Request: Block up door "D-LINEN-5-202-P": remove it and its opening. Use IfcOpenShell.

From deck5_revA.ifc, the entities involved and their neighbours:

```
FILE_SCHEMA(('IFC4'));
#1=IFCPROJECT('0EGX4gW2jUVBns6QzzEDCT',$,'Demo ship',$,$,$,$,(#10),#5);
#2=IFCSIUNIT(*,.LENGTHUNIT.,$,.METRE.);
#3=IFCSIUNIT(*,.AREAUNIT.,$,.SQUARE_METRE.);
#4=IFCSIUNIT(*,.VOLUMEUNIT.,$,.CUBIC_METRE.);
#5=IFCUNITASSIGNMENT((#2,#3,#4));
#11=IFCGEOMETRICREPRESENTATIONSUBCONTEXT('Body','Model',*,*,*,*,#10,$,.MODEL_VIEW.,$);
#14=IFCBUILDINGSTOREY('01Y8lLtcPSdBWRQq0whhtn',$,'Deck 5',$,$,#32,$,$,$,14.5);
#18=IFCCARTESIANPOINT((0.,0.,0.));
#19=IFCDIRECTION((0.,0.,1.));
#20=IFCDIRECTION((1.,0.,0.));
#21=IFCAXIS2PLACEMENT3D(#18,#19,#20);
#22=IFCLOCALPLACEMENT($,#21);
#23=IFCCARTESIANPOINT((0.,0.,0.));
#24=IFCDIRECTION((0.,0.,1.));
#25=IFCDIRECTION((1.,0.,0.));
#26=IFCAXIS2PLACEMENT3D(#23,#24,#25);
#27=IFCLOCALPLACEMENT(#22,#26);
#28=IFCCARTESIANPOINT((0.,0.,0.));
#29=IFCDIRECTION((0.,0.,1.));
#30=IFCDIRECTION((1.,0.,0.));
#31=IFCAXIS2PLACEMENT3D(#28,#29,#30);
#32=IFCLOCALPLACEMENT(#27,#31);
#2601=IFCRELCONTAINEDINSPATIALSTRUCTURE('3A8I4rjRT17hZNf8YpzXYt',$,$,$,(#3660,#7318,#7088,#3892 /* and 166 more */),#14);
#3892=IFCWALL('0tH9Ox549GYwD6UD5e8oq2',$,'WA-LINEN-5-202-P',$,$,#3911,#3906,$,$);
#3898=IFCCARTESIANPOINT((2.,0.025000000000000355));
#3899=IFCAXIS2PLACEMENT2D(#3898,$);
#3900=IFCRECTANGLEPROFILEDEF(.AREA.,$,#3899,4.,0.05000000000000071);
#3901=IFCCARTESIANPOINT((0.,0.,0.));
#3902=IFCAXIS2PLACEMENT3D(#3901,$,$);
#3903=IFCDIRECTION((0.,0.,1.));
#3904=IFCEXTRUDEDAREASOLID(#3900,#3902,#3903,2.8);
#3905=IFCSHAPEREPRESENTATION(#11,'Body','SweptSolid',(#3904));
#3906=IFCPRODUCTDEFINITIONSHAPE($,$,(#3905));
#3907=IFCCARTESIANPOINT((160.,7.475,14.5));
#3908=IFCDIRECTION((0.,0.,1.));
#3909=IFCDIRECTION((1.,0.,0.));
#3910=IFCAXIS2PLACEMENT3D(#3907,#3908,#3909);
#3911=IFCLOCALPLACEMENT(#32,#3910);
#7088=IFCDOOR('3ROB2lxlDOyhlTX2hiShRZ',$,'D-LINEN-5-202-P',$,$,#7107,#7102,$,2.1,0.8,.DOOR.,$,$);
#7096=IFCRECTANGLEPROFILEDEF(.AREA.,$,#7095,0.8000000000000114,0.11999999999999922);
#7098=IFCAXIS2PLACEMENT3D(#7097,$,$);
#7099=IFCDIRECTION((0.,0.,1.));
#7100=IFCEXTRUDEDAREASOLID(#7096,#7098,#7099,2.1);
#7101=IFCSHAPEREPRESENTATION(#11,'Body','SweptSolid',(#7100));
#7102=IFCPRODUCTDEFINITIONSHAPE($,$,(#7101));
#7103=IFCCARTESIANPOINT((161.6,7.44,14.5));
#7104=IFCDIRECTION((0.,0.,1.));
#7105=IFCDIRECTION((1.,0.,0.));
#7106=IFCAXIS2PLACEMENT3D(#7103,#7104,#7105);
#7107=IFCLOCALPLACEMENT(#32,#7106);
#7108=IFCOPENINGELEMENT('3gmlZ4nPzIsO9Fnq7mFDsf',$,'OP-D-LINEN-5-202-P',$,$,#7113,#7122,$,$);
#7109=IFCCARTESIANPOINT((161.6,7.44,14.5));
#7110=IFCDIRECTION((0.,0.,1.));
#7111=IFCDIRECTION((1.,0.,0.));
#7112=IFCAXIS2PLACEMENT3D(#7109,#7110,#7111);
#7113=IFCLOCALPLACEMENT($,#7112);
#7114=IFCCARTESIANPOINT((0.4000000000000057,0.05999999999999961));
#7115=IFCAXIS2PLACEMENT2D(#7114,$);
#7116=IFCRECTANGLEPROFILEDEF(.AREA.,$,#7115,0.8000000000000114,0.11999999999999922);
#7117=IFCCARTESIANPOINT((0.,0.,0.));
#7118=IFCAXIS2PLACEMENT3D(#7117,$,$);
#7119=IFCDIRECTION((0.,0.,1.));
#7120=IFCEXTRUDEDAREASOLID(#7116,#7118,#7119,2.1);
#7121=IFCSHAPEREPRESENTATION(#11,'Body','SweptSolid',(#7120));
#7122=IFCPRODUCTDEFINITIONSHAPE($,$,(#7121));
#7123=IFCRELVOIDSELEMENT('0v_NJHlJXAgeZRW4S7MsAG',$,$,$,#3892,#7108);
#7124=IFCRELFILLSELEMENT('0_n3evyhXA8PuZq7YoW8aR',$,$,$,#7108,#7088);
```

```python
import ifcopenshell
import ifcopenshell.api.feature
import ifcopenshell.api.root
import ifcopenshell.geom
import ifcopenshell.util.shape

model = ifcopenshell.open("deck5_revA.ifc")
settings = ifcopenshell.geom.settings()


def volume(element):
    """Net volume in cubic metres, openings subtracted."""
    shape = ifcopenshell.geom.create_shape(settings, element)
    return ifcopenshell.util.shape.get_volume(shape.geometry)


door = model.by_guid("3ROB2lxlDOyhlTX2hiShRZ")
opening = door.FillsVoids[0].RelatingOpeningElement
wall = opening.VoidsElements[0].RelatingBuildingElement
before = volume(wall)

ifcopenshell.api.root.remove_product(model, product=door)
ifcopenshell.api.feature.remove_feature(model, feature=opening)

after = volume(wall)

print(f"wall volume {before:.3f} -> {after:.3f} m3")

model.write("deck5_revA-out.ifc")
```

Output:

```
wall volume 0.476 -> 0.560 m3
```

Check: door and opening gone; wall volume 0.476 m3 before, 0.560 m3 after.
